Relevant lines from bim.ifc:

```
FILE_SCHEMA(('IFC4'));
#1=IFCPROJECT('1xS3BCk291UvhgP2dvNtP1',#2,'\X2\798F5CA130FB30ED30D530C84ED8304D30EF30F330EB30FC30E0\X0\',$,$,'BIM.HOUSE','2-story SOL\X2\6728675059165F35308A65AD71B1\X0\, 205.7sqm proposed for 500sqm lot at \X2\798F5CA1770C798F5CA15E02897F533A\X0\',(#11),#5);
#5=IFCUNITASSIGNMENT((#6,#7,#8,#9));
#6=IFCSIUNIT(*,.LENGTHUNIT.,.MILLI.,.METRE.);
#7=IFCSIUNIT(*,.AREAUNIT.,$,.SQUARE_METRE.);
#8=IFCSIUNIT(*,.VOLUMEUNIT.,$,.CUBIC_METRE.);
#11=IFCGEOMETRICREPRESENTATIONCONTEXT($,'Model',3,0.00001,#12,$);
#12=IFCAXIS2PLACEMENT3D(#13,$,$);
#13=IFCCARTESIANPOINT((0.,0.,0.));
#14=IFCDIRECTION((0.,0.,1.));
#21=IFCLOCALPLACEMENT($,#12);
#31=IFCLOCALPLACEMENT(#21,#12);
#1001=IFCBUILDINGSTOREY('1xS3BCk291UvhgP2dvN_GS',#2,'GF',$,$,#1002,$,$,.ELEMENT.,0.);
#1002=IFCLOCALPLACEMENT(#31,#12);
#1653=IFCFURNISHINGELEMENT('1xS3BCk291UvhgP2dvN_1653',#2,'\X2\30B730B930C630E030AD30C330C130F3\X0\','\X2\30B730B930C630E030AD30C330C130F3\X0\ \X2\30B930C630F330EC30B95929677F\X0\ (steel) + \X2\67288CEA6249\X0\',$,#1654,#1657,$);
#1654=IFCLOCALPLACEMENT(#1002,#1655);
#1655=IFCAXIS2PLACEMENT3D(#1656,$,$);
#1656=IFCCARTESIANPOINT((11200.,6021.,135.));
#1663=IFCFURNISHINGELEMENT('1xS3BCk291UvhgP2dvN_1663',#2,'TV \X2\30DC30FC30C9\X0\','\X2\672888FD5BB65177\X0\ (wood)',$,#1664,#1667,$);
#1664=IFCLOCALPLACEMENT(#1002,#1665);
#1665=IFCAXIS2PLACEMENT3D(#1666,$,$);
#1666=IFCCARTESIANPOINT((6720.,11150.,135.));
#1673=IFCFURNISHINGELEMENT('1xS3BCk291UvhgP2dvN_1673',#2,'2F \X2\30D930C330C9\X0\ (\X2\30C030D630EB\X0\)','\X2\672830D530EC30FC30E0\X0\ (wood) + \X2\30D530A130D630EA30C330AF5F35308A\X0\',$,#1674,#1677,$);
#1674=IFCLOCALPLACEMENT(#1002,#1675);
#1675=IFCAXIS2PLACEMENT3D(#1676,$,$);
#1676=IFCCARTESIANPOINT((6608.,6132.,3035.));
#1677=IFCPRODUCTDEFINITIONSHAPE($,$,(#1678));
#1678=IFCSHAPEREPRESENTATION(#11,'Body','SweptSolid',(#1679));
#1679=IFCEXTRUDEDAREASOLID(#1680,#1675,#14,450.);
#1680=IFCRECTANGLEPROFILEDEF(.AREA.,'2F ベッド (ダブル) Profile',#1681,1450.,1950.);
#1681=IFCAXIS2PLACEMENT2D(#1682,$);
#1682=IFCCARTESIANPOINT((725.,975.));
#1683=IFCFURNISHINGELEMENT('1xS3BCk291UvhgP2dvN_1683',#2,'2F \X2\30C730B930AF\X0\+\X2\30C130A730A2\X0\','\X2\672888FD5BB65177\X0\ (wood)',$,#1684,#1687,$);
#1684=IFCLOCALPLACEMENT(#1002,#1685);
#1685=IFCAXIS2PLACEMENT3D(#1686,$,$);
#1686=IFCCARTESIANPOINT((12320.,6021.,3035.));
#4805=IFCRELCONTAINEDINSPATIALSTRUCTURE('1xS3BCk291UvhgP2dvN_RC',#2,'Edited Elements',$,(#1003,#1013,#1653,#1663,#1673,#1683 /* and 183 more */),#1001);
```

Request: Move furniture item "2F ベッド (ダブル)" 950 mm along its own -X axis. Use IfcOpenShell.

```python
import ifcopenshell
import ifcopenshell.api.geometry
import ifcopenshell.util.placement

model = ifcopenshell.open("bim.ifc")

item = model.by_guid("1xS3BCk291UvhgP2dvN_1673")
matrix = ifcopenshell.util.placement.get_local_placement(item.ObjectPlacement)
matrix[:3, 3] -= matrix[:3, 0] * 950.0
ifcopenshell.api.geometry.edit_object_placement(model, product=item, matrix=matrix, is_si=False)

print(ifcopenshell.util.placement.get_local_placement(item.ObjectPlacement).round(3) + 0.0)

model.write("bim_v2.ifc")
```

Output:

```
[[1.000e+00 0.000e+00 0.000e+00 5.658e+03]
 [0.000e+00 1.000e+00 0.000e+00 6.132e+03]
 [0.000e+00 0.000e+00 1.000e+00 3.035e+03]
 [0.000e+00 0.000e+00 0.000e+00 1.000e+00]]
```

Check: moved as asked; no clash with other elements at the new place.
